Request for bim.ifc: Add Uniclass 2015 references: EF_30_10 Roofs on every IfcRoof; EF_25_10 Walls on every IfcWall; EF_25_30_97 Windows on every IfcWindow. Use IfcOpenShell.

First a look at what the model holds.

```python
import ifcopenshell

model = ifcopenshell.open("bim.ifc")
print(model.schema)
print("classifications:", [c.Name for c in model.by_type("IfcClassification")])
for ifc_class in ("IfcDoor", "IfcRoof", "IfcStair", "IfcWall", "IfcWindow"):
    print(ifc_class, len(model.by_type(ifc_class)))
```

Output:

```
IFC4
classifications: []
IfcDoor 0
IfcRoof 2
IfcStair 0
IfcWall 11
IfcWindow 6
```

```python
import ifcopenshell
import ifcopenshell.api.classification

model = ifcopenshell.open("bim.ifc")

system = ifcopenshell.api.classification.add_classification(model, classification="Uniclass 2015")

codes = {
    "IfcRoof": ("EF_30_10", "Roofs"),
    "IfcWall": ("EF_25_10", "Walls"),
    "IfcWindow": ("EF_25_30_97", "Windows"),
}
for ifc_class, (code, name) in codes.items():
    products = model.by_type(ifc_class)
    ifcopenshell.api.classification.add_reference(
        model, products=products, classification=system, identification=code, name=name
    )
    print(code, len(products))

model.write("bim_v2.ifc")
```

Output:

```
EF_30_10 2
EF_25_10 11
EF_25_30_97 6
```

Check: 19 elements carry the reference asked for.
